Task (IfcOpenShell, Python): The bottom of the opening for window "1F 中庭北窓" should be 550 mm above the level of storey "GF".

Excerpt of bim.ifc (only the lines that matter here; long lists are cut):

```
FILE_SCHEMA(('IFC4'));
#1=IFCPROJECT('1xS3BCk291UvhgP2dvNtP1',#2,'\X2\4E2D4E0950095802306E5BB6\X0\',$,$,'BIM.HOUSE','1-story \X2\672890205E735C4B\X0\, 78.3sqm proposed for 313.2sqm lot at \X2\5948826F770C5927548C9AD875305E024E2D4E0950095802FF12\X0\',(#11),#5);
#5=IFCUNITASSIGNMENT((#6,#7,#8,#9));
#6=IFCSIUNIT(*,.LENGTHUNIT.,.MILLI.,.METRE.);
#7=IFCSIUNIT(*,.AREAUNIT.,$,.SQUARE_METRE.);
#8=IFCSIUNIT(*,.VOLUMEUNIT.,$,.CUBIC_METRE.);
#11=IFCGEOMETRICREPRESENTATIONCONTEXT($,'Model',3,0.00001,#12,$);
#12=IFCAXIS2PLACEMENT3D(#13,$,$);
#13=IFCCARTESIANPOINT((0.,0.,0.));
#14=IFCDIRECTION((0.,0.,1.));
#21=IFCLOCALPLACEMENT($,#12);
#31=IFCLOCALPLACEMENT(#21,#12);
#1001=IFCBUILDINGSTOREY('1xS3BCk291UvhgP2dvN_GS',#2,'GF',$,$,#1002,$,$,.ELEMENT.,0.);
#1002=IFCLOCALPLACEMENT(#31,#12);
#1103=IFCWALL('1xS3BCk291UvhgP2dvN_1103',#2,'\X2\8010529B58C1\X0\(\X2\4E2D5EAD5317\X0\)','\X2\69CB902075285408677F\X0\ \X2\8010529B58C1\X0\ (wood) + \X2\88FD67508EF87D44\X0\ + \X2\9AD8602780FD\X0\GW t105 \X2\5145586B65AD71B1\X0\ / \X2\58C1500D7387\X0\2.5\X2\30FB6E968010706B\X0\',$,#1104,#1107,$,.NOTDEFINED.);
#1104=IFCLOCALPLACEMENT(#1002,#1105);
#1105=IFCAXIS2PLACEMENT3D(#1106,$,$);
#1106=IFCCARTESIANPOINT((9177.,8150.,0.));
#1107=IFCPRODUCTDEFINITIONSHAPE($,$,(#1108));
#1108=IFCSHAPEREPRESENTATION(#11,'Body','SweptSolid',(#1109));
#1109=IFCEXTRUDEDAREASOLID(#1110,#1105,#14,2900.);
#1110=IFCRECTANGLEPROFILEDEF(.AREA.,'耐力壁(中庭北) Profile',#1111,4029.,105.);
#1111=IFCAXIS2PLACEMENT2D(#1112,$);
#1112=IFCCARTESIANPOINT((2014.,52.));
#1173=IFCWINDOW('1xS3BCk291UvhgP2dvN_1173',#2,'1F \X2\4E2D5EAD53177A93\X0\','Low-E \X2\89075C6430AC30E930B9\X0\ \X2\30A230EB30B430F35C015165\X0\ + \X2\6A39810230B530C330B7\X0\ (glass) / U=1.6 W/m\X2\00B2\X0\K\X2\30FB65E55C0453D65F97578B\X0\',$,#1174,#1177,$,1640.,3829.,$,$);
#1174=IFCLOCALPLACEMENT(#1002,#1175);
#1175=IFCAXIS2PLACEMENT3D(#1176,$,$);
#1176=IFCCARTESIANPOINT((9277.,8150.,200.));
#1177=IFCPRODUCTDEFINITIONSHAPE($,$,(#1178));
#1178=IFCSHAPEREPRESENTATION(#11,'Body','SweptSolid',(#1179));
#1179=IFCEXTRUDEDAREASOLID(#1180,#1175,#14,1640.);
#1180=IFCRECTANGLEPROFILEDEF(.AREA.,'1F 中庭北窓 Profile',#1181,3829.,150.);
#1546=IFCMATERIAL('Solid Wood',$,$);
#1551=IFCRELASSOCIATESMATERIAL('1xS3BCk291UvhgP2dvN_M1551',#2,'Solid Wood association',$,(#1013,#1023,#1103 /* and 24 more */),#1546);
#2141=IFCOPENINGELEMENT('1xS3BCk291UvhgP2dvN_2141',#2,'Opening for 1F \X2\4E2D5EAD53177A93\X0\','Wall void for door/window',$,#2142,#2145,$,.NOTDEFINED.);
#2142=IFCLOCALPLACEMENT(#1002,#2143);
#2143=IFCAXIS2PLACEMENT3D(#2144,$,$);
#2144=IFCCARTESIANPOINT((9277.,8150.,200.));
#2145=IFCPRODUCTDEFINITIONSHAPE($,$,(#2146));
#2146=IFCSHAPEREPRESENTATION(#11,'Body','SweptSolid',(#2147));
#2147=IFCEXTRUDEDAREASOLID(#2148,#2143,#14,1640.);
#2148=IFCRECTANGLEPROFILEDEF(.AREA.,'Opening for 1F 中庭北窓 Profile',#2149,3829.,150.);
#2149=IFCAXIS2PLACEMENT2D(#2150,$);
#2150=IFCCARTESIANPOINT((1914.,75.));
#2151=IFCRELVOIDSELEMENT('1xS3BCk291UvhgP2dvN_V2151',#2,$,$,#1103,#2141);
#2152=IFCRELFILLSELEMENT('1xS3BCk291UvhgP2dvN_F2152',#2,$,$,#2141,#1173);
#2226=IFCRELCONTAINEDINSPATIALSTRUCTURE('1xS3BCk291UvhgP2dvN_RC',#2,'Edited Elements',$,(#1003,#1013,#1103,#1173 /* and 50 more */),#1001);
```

```python
import numpy as np
import ifcopenshell
import ifcopenshell.api.geometry
import ifcopenshell.geom
import ifcopenshell.util.element
import ifcopenshell.util.placement
import ifcopenshell.util.shape
import ifcopenshell.util.unit

model = ifcopenshell.open("bim.ifc")
unit_scale = ifcopenshell.util.unit.calculate_unit_scale(model)

window = model.by_guid("1xS3BCk291UvhgP2dvN_1173")
opening = window.FillsVoids[0].RelatingOpeningElement
storey = ifcopenshell.util.element.get_container(window, ifc_class="IfcBuildingStorey")
level = ifcopenshell.util.placement.get_local_placement(storey.ObjectPlacement)[2, 3]

# The opening's origin need not be at the sill, so measure its lowest point.
shape = ifcopenshell.geom.create_shape(ifcopenshell.geom.settings(), opening)
bottom = ifcopenshell.util.shape.get_shape_bottom_elevation(shape, shape.geometry) / unit_scale
dz = level + 0.55 / unit_scale - bottom

shift = np.array([0.0, 0.0, dz])
# The window is not placed relative to its opening, so move both.
for product in (opening, window):
    matrix = ifcopenshell.util.placement.get_local_placement(product.ObjectPlacement)
    matrix[:3, 3] += shift
    ifcopenshell.api.geometry.edit_object_placement(model, product=product, matrix=matrix, is_si=False)

print(f"moved by {dz * unit_scale:+.3f} m")

model.write("bim-out.ifc")
```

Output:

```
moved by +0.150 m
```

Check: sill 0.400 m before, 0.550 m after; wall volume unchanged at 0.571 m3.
